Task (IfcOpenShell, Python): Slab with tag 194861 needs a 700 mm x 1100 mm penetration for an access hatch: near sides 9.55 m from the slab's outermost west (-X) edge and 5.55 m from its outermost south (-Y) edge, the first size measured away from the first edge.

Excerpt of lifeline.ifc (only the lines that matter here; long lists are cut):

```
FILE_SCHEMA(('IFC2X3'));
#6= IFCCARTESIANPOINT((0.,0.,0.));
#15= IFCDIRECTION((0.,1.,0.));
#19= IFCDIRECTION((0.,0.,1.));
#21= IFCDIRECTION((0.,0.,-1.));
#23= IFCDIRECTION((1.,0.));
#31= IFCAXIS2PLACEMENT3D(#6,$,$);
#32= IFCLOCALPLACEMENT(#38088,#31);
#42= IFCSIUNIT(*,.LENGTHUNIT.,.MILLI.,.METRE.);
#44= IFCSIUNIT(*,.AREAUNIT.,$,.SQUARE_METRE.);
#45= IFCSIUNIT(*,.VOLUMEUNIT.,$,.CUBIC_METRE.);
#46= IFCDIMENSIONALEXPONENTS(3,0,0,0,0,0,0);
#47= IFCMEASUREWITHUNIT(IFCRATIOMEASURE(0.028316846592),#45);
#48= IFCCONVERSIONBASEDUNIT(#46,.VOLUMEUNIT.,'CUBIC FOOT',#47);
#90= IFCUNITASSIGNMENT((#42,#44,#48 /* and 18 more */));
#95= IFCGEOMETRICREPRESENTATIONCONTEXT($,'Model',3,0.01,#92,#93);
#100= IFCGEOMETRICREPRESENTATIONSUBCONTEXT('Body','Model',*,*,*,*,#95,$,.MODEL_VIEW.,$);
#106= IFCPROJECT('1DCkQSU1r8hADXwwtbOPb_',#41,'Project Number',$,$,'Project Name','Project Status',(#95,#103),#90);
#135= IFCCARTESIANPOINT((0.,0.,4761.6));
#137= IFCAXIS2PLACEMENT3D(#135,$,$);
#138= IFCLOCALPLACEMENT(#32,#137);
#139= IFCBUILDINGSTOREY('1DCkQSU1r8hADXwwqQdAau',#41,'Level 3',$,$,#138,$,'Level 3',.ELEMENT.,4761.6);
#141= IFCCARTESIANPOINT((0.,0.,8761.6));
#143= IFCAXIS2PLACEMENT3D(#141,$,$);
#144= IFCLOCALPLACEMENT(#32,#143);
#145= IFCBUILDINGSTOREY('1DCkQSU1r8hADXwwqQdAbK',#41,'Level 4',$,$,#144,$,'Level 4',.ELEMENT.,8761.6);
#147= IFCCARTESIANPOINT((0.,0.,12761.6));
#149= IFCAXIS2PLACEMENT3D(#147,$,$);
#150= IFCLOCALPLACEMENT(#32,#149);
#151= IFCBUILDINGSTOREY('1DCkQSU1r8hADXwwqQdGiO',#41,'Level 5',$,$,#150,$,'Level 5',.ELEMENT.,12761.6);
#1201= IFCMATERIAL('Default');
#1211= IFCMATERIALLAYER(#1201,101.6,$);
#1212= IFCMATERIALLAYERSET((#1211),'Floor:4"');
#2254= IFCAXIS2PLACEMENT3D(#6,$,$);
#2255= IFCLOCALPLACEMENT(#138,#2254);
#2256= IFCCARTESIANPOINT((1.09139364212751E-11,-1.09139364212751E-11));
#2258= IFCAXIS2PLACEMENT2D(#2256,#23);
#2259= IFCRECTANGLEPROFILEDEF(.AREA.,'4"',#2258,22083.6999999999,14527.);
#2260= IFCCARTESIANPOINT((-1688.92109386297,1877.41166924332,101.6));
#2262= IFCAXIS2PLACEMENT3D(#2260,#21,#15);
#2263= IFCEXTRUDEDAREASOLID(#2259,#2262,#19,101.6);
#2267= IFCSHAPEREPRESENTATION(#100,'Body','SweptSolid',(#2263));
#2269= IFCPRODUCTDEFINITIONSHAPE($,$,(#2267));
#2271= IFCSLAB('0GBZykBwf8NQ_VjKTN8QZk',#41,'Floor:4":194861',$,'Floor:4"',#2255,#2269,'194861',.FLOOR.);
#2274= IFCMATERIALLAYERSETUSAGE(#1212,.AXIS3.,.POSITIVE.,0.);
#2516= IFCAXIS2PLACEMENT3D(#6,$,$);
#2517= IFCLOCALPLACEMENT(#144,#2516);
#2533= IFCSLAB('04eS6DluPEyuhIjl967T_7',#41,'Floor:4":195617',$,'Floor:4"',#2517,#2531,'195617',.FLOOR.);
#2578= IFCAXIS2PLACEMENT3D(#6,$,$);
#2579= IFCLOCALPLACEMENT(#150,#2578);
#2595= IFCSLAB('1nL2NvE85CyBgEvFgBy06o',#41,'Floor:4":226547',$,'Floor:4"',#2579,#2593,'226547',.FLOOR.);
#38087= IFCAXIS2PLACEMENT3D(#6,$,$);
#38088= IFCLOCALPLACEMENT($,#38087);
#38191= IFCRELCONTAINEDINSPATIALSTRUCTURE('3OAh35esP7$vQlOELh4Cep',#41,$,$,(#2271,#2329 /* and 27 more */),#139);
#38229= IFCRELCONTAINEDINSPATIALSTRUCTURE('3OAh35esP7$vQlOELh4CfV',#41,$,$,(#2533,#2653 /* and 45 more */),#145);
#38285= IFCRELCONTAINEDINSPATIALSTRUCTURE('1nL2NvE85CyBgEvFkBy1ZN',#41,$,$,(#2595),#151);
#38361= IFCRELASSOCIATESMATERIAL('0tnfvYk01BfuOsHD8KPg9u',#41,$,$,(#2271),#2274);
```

```python
import numpy as np
import ifcopenshell
import ifcopenshell.api.feature
import ifcopenshell.api.geometry
import ifcopenshell.api.root
import ifcopenshell.geom
import ifcopenshell.util.placement
import ifcopenshell.util.representation
import ifcopenshell.util.shape
import ifcopenshell.util.unit

model = ifcopenshell.open("lifeline.ifc")
unit_scale = ifcopenshell.util.unit.calculate_unit_scale(model)
settings = ifcopenshell.geom.settings()


def volume(element):
    """Net volume in cubic metres, openings subtracted."""
    shape = ifcopenshell.geom.create_shape(settings, element)
    return ifcopenshell.util.shape.get_volume(shape.geometry)


slab = model.by_guid("0GBZykBwf8NQ_VjKTN8QZk")
before = volume(slab)

# Extent in the slab's own axes, in metres. The edges named are its -X and -Y sides.
slab_shape = ifcopenshell.geom.create_shape(settings, slab)
vertices = ifcopenshell.util.shape.get_vertices(slab_shape.geometry)
x_min, y_min, bottom = vertices.min(axis=0)
top = vertices[:, 2].max()

opening = ifcopenshell.api.root.create_entity(model, ifc_class="IfcOpeningElement", name="Access hatch opening")
context = ifcopenshell.util.representation.get_context(model, "Model", "Body", "MODEL_VIEW")
width, depth = 0.7, 1.1
outline = [(0.0, 0.0), (width, 0.0), (width, depth), (0.0, depth), (0.0, 0.0)]
# Overshoot both faces by 50 mm so the cut is clean.
shape = ifcopenshell.api.geometry.add_slab_representation(
    model, context=context, depth=top - bottom + 0.1, polyline=outline
)
ifcopenshell.api.geometry.assign_representation(model, product=opening, representation=shape)

matrix = ifcopenshell.util.placement.get_local_placement(slab.ObjectPlacement)
matrix[:, 3] = matrix @ np.append(np.array([x_min + 9.55, y_min + 5.55, bottom - 0.05]) / unit_scale, 1.0)
ifcopenshell.api.geometry.edit_object_placement(model, product=opening, matrix=matrix, is_si=False)
ifcopenshell.api.feature.add_feature(model, feature=opening, element=slab)

after = volume(slab)

print(f"slab volume {before:.3f} -> {after:.3f} m3")

model.write("lifeline_updated.ifc")
```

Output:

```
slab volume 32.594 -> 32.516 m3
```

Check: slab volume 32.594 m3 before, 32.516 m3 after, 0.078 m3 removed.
